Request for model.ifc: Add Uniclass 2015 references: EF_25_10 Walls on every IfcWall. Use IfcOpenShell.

First a look at what the model holds.

```python
import ifcopenshell

model = ifcopenshell.open("model.ifc")
print(model.schema)
print("classifications:", [c.Name for c in model.by_type("IfcClassification")])
for ifc_class in ("IfcDoor", "IfcRoof", "IfcStair", "IfcWall", "IfcWindow"):
    print(ifc_class, len(model.by_type(ifc_class)))
```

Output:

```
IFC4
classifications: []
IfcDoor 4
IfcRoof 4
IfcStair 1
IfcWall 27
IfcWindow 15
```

```python
import ifcopenshell
import ifcopenshell.api.classification

model = ifcopenshell.open("model.ifc")

system = ifcopenshell.api.classification.add_classification(model, classification="Uniclass 2015")

codes = {
    "IfcWall": ("EF_25_10", "Walls"),
}
for ifc_class, (code, name) in codes.items():
    products = model.by_type(ifc_class)
    ifcopenshell.api.classification.add_reference(
        model, products=products, classification=system, identification=code, name=name
    )
    print(code, len(products))

model.write("model-out.ifc")
```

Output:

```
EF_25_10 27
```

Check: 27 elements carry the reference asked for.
